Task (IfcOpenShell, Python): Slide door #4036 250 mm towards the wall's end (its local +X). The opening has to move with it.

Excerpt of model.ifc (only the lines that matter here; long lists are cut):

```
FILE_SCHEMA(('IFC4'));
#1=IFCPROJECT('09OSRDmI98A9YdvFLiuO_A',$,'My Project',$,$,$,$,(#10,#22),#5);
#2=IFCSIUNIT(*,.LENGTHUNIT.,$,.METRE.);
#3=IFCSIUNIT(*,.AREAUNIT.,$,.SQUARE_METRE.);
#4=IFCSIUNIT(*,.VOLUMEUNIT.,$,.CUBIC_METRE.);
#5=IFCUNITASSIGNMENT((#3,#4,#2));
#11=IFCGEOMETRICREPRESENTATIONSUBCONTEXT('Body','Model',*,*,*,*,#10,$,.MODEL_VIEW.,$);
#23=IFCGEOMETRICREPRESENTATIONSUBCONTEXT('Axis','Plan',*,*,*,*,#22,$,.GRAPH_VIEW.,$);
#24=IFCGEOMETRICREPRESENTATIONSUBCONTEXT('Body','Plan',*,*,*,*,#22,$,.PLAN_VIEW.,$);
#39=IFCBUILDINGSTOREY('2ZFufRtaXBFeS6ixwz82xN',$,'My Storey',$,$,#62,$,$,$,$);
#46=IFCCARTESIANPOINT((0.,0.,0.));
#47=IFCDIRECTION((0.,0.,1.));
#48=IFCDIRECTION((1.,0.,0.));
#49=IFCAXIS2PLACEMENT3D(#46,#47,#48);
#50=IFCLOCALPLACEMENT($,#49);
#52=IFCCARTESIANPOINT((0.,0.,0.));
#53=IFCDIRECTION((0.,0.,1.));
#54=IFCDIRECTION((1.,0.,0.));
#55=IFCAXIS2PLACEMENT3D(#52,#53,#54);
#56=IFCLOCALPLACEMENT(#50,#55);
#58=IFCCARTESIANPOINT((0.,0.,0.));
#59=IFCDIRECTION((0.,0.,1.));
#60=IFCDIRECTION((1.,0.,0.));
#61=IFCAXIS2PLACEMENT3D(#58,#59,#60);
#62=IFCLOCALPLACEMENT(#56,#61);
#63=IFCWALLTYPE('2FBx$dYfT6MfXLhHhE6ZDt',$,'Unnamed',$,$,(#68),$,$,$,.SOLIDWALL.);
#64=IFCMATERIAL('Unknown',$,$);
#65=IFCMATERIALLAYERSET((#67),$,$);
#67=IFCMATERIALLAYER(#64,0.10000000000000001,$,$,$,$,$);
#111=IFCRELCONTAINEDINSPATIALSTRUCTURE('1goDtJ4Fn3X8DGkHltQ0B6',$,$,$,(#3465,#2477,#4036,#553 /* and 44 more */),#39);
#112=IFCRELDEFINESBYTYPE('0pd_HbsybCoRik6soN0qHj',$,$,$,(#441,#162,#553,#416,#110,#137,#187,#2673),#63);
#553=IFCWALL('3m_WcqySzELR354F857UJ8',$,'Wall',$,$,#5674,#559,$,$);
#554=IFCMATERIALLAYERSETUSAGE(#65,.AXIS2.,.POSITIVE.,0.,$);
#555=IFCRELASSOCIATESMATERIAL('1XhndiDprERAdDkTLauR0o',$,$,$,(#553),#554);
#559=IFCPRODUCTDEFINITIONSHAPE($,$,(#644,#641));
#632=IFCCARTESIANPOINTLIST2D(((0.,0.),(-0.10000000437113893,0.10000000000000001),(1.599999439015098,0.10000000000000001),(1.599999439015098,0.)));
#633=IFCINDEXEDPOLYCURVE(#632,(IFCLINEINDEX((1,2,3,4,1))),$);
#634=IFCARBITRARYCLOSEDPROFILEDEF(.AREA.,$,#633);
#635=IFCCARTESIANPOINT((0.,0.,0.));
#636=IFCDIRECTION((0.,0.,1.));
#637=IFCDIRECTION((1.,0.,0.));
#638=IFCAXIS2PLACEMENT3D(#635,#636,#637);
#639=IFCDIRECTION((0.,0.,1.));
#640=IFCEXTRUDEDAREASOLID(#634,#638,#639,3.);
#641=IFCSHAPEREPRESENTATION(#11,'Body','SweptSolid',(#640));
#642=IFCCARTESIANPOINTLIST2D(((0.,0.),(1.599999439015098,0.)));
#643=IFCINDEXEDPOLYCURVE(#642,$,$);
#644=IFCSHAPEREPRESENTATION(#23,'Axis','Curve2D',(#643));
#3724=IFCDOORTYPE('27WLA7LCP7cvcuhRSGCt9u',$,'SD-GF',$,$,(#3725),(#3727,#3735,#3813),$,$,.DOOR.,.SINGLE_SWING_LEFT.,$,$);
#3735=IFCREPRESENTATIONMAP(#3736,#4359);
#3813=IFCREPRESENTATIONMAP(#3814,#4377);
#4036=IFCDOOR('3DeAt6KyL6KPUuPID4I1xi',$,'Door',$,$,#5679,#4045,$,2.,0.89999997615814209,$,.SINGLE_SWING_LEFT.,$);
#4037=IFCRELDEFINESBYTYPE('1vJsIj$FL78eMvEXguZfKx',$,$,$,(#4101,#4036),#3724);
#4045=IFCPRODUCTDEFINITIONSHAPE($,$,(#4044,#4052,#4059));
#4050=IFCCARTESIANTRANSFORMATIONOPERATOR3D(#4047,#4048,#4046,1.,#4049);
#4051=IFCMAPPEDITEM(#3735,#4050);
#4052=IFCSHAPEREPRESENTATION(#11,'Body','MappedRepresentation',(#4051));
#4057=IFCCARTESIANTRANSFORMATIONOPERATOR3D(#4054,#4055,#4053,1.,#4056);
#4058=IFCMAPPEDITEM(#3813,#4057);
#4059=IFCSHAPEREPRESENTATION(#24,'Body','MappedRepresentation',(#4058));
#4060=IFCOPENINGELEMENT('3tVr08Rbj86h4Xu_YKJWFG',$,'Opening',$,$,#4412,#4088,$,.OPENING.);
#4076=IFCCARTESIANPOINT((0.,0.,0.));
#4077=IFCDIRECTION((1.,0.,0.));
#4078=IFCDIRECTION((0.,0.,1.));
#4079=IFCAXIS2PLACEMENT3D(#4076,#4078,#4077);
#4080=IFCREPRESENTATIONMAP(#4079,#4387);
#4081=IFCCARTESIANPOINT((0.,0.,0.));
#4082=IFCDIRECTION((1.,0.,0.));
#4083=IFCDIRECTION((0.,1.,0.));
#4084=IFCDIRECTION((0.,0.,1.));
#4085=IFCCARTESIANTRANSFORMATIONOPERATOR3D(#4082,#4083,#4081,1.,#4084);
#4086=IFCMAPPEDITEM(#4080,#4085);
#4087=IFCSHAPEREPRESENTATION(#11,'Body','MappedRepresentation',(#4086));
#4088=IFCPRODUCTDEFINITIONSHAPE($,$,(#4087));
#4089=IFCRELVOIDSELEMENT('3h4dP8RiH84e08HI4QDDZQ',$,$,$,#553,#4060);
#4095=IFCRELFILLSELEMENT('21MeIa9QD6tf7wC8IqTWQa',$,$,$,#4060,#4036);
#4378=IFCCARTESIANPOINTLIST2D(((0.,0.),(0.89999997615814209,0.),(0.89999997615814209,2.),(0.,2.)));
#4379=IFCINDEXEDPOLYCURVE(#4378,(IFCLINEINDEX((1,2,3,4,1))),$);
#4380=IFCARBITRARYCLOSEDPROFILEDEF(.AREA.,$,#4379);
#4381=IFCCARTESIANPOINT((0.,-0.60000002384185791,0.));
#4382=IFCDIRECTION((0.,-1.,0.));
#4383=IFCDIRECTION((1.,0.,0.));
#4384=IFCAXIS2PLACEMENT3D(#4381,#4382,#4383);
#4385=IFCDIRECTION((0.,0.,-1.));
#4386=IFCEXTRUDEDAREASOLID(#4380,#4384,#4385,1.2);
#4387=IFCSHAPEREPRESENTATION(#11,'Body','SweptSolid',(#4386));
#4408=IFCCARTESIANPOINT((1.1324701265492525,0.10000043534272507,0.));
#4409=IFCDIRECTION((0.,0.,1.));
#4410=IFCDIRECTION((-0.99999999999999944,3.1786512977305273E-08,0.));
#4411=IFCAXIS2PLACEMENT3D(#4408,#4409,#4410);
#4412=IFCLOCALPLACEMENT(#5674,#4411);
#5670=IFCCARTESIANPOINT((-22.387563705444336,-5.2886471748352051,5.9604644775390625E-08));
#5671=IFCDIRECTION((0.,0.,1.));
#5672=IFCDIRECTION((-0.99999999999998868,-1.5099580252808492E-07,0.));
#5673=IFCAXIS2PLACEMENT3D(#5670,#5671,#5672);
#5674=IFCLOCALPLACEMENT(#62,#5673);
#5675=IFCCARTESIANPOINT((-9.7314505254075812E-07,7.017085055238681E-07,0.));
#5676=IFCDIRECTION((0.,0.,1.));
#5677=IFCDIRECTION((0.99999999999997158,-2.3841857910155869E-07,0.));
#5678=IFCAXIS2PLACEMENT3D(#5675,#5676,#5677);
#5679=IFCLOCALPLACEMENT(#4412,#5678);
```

```python
import ifcopenshell
import ifcopenshell.api.geometry
import ifcopenshell.util.placement

model = ifcopenshell.open("model.ifc")

door = model.by_guid("3DeAt6KyL6KPUuPID4I1xi")
opening = door.FillsVoids[0].RelatingOpeningElement
wall = opening.VoidsElements[0].RelatingBuildingElement

wall_matrix = ifcopenshell.util.placement.get_local_placement(wall.ObjectPlacement)
shift = wall_matrix[:3, 0] * 0.25
before = ifcopenshell.util.placement.get_local_placement(door.ObjectPlacement)[:3, 3].copy()

# The door is placed relative to its opening, so it follows when the opening moves.
matrix = ifcopenshell.util.placement.get_local_placement(opening.ObjectPlacement)
matrix[:3, 3] += shift
ifcopenshell.api.geometry.edit_object_placement(
    model, product=opening, matrix=matrix, is_si=False, should_transform_children=True
)

after = ifcopenshell.util.placement.get_local_placement(door.ObjectPlacement)[:3, 3]
print("door moved by", (after - before).round(3) + 0.0)

model.write("model_v2.ifc")
```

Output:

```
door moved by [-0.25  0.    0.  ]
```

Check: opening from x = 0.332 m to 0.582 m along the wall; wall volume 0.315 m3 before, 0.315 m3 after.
